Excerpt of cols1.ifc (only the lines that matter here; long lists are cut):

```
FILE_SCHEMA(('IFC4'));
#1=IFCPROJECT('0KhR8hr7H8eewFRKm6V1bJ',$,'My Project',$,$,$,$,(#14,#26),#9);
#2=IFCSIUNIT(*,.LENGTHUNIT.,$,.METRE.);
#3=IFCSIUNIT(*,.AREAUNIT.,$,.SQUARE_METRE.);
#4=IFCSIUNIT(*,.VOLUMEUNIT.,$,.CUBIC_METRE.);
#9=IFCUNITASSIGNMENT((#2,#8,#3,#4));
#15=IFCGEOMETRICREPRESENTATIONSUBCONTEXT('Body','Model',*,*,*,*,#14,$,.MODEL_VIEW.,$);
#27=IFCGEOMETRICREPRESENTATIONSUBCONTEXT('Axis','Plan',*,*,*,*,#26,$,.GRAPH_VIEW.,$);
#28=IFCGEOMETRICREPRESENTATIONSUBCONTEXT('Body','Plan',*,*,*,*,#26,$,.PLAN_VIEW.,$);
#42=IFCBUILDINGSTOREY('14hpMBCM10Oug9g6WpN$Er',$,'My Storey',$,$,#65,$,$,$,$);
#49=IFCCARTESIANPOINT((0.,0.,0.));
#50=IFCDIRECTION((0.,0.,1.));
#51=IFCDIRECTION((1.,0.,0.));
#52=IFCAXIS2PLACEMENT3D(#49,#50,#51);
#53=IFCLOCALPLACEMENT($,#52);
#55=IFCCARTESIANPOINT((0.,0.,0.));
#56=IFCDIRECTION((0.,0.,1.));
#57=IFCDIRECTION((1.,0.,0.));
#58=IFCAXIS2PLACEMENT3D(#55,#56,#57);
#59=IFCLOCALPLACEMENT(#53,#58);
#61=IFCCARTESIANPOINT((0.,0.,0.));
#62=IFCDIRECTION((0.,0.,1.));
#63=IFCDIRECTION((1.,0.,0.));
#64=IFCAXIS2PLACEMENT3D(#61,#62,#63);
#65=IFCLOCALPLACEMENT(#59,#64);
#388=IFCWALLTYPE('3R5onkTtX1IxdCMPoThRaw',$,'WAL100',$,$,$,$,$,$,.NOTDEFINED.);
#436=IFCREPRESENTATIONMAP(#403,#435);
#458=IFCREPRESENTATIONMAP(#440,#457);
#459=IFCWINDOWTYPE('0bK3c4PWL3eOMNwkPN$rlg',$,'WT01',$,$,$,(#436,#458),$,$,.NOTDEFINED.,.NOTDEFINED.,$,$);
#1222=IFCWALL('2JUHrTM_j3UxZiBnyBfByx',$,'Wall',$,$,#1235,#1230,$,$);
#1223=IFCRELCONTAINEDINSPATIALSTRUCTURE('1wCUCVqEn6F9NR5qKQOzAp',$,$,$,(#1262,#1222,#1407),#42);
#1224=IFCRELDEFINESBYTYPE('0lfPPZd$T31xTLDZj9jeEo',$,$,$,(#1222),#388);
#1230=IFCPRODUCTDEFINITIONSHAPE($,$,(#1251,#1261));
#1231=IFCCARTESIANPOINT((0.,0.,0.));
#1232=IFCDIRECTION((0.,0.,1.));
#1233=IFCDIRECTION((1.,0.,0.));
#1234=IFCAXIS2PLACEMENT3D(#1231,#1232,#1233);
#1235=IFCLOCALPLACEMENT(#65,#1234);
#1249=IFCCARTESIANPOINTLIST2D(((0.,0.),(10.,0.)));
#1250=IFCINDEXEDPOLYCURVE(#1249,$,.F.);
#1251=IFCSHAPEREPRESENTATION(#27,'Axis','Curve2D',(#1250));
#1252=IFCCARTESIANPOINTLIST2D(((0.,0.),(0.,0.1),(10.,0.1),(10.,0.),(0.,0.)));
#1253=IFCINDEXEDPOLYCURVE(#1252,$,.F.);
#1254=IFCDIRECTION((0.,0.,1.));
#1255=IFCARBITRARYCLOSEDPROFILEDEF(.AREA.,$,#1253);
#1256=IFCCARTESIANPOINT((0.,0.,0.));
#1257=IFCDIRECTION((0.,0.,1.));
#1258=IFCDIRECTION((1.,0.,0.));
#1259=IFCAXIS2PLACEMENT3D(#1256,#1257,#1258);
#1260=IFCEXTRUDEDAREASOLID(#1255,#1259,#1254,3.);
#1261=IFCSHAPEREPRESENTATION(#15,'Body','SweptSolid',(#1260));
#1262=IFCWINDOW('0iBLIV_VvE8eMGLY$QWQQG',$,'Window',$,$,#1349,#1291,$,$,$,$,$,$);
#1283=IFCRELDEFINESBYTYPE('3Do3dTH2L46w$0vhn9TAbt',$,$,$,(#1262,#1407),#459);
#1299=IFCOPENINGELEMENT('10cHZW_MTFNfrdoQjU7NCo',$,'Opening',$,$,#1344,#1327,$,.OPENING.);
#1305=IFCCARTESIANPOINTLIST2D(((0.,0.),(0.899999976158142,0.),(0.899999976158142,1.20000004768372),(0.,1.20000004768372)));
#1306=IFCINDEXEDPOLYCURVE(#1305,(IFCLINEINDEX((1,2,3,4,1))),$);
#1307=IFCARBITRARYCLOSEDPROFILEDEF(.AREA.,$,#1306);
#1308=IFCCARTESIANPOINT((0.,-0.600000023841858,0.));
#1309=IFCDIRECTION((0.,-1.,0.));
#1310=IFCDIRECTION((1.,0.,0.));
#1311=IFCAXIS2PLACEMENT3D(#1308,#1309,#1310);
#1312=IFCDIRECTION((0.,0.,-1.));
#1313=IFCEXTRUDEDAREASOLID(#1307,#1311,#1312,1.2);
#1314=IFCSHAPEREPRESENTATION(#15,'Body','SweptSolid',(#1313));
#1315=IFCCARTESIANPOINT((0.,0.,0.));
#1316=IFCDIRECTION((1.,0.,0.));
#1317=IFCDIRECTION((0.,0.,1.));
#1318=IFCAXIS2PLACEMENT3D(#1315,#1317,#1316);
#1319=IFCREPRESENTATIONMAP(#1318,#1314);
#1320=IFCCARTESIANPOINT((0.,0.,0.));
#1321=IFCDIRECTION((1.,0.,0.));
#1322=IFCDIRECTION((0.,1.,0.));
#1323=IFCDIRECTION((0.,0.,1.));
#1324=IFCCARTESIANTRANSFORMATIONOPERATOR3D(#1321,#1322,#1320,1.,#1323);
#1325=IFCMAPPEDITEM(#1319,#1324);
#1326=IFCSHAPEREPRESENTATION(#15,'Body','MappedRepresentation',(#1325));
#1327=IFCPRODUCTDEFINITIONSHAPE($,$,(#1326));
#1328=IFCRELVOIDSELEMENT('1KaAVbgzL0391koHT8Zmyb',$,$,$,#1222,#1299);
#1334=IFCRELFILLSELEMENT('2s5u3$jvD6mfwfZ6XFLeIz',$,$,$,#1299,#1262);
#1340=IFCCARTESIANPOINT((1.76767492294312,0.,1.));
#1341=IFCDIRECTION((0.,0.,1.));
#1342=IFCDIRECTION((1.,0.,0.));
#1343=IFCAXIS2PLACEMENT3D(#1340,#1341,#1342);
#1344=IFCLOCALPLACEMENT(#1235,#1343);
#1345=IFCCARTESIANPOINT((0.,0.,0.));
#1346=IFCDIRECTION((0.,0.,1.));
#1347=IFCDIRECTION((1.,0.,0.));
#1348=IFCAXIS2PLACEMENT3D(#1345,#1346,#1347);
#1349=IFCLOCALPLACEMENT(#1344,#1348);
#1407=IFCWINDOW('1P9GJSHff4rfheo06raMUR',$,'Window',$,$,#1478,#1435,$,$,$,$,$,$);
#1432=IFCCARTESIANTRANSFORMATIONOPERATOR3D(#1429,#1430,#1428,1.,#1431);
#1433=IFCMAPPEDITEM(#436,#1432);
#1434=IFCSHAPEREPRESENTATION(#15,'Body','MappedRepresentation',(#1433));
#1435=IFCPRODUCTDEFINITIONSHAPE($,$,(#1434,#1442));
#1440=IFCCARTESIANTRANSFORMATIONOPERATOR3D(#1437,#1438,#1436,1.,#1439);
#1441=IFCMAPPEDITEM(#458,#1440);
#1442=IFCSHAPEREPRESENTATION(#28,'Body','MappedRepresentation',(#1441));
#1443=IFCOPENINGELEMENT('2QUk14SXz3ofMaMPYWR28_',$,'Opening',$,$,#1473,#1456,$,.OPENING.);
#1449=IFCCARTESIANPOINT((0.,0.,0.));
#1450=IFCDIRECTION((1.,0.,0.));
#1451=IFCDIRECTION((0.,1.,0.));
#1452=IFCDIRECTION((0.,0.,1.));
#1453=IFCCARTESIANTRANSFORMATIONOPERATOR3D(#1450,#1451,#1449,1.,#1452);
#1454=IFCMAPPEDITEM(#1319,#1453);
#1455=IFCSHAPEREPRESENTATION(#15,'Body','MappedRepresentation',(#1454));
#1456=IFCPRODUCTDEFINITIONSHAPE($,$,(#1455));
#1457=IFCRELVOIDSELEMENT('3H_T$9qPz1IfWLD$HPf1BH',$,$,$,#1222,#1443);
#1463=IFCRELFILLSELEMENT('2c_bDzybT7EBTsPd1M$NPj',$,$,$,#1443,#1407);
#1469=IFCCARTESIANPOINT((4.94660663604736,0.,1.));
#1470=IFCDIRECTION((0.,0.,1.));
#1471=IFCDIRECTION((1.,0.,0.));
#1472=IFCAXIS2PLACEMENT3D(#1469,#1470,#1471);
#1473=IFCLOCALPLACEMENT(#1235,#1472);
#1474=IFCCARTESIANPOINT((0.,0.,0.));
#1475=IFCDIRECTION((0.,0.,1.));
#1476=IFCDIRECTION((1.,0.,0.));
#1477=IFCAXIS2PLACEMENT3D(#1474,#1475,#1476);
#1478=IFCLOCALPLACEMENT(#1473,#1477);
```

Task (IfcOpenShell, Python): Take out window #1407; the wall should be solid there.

```python
import ifcopenshell
import ifcopenshell.api.feature
import ifcopenshell.api.root
import ifcopenshell.geom
import ifcopenshell.util.shape

model = ifcopenshell.open("cols1.ifc")
settings = ifcopenshell.geom.settings()


def volume(element):
    """Net volume in cubic metres, openings subtracted."""
    shape = ifcopenshell.geom.create_shape(settings, element)
    return ifcopenshell.util.shape.get_volume(shape.geometry)


window = model.by_guid("1P9GJSHff4rfheo06raMUR")
opening = window.FillsVoids[0].RelatingOpeningElement
wall = opening.VoidsElements[0].RelatingBuildingElement
before = volume(wall)

ifcopenshell.api.root.remove_product(model, product=window)
ifcopenshell.api.feature.remove_feature(model, feature=opening)

after = volume(wall)

print(f"wall volume {before:.3f} -> {after:.3f} m3")

model.write("cols1_edited.ifc")
```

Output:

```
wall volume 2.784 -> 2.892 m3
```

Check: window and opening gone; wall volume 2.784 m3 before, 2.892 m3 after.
